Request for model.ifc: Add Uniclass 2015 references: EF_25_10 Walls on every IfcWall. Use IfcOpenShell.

First a look at what the model holds.

```python
import ifcopenshell

model = ifcopenshell.open("model.ifc")
print(model.schema)
print("classifications:", [c.Name for c in model.by_type("IfcClassification")])
for ifc_class in ("IfcDoor", "IfcRoof", "IfcStair", "IfcWall", "IfcWindow"):
    print(ifc_class, len(model.by_type(ifc_class)))
```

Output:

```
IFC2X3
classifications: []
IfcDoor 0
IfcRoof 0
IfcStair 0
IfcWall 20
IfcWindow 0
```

```python
import ifcopenshell
import ifcopenshell.api.classification

model = ifcopenshell.open("model.ifc")

# IFC2X3 requires Source and Edition and has no link from the project to the system.
system = model.create_entity("IfcClassification", Source="NBS", Edition="2015", Name="Uniclass 2015")

codes = {
    "IfcWall": ("EF_25_10", "Walls"),
}
for ifc_class, (code, name) in codes.items():
    products = model.by_type(ifc_class)
    ifcopenshell.api.classification.add_reference(
        model, products=products, classification=system, identification=code, name=name
    )
    print(code, len(products))

model.write("model_rev.ifc")
```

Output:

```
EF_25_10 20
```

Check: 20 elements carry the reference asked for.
